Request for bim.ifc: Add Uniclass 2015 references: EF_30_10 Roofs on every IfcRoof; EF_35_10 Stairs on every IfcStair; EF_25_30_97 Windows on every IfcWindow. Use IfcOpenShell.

First a look at what the model holds.

```python
import ifcopenshell

model = ifcopenshell.open("bim.ifc")
print(model.schema)
print("classifications:", [c.Name for c in model.by_type("IfcClassification")])
for ifc_class in ("IfcDoor", "IfcRoof", "IfcStair", "IfcWall", "IfcWindow"):
    print(ifc_class, len(model.by_type(ifc_class)))
```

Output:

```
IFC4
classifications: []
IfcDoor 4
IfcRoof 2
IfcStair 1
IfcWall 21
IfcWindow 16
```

```python
import ifcopenshell
import ifcopenshell.api.classification

model = ifcopenshell.open("bim.ifc")

system = ifcopenshell.api.classification.add_classification(model, classification="Uniclass 2015")

codes = {
    "IfcRoof": ("EF_30_10", "Roofs"),
    "IfcStair": ("EF_35_10", "Stairs"),
    "IfcWindow": ("EF_25_30_97", "Windows"),
}
for ifc_class, (code, name) in codes.items():
    products = model.by_type(ifc_class)
    ifcopenshell.api.classification.add_reference(
        model, products=products, classification=system, identification=code, name=name
    )
    print(code, len(products))

model.write("bim_updated.ifc")
```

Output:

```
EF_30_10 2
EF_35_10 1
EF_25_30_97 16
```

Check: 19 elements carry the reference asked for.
